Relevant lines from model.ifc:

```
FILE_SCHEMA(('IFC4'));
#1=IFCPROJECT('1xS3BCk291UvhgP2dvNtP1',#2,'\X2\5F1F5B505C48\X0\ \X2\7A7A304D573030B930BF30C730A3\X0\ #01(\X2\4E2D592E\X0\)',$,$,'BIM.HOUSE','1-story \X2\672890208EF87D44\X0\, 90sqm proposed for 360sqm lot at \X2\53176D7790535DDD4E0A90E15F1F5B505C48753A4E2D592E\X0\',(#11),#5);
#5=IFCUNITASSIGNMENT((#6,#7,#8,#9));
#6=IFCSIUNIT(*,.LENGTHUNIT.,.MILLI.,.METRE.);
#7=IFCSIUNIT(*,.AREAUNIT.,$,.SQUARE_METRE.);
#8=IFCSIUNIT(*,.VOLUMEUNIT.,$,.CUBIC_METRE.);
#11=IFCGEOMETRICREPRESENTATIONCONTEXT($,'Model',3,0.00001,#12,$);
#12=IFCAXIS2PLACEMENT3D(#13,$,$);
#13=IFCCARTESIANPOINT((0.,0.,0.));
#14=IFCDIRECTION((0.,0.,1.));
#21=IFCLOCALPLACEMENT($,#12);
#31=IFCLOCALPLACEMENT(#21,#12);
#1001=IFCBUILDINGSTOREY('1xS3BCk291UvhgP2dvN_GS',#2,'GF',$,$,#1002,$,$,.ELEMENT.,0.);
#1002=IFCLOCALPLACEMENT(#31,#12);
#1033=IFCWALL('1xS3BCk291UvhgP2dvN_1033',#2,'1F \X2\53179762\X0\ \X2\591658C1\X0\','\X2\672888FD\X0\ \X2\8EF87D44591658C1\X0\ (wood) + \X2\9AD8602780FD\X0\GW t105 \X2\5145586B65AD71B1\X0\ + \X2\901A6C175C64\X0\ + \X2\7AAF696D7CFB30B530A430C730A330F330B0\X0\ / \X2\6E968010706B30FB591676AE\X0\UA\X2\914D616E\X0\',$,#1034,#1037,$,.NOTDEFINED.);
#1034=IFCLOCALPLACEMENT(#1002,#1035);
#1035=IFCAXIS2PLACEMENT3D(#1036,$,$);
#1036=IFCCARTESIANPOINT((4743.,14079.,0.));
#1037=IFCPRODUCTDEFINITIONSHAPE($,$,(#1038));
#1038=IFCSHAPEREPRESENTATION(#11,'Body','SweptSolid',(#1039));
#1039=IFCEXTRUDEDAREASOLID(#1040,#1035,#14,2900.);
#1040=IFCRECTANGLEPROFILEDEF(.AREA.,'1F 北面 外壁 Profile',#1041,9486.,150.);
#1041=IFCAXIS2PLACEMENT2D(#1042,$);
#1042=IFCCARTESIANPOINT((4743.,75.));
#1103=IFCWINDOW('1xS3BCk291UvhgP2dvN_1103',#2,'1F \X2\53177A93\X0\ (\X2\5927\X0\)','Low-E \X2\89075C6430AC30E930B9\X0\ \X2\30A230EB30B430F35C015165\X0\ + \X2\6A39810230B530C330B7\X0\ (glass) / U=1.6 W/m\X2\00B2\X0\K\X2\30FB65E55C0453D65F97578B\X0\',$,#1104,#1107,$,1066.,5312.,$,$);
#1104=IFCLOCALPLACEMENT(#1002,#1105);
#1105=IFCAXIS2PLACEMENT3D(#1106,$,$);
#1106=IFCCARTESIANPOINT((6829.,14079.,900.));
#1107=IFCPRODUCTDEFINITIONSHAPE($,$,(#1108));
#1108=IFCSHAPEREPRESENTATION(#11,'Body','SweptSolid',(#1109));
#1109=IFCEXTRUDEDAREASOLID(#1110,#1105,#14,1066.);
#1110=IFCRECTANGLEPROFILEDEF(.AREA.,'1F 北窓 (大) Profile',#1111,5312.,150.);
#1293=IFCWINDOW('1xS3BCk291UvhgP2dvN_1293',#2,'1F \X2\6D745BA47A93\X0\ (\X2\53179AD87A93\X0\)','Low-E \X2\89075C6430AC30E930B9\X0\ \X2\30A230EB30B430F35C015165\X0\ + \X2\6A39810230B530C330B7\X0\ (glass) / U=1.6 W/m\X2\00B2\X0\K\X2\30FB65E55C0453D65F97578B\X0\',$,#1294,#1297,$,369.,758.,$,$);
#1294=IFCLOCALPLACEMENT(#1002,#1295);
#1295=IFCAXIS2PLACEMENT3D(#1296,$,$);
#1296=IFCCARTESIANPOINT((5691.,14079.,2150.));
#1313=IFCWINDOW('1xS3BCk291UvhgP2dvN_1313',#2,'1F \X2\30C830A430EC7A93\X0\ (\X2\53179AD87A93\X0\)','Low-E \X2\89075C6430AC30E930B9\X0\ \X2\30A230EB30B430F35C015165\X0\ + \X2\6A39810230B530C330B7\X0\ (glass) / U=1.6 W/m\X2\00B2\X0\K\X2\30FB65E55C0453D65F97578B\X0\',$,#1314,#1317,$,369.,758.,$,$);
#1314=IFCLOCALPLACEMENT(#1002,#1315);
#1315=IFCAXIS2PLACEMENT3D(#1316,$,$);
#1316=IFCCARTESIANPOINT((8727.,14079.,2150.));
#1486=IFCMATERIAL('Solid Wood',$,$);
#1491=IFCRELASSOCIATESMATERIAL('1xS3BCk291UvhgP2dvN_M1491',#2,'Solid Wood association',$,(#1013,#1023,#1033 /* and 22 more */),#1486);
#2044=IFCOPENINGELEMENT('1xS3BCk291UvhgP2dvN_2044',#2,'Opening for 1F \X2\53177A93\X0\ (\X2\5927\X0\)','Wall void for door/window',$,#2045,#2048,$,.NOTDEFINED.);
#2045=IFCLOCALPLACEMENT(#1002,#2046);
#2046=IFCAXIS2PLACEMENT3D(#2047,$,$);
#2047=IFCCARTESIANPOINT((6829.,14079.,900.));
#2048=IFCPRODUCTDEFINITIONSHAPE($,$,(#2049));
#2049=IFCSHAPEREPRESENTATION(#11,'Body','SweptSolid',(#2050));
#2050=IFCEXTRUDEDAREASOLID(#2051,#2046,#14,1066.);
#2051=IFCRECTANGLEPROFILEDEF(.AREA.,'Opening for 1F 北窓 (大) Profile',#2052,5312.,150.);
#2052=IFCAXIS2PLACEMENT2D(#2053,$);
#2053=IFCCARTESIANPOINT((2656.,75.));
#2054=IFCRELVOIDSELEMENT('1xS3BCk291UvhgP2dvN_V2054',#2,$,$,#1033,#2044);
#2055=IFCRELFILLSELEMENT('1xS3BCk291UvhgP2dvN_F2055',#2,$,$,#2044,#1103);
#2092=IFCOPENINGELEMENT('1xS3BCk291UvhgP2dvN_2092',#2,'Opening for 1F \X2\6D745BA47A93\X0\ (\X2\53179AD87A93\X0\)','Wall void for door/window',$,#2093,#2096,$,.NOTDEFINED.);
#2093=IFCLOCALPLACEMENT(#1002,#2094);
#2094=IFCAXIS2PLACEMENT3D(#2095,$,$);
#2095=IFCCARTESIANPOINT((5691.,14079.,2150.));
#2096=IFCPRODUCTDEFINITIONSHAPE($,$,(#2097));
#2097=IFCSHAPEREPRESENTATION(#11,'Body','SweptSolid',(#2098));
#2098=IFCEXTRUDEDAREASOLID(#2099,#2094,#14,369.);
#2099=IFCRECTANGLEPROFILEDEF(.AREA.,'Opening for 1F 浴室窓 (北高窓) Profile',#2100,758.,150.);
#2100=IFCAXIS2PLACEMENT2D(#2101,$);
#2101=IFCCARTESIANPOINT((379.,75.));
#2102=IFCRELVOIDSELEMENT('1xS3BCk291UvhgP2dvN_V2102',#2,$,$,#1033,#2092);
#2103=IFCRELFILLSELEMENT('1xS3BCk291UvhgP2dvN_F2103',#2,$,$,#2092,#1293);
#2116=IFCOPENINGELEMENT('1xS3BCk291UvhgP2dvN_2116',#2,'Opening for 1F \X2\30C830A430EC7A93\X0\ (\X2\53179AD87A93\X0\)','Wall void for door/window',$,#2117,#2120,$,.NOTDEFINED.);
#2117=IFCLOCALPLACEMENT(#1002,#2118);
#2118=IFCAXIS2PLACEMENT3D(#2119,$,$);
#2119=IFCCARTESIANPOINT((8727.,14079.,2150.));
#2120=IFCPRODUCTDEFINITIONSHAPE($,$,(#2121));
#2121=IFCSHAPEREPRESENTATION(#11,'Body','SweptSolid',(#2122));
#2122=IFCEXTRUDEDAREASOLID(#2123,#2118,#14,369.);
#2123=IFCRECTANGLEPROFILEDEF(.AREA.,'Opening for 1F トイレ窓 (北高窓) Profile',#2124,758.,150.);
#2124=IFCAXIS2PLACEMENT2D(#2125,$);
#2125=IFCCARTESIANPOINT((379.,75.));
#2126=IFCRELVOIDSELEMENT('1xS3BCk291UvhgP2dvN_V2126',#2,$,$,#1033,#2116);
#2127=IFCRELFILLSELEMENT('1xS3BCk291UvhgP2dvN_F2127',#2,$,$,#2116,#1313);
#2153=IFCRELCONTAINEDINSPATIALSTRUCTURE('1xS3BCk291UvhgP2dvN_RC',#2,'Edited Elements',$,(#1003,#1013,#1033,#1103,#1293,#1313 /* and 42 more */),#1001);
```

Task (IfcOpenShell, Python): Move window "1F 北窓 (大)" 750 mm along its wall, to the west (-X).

```python
import ifcopenshell
import ifcopenshell.api.geometry
import ifcopenshell.util.placement
import ifcopenshell.util.unit

model = ifcopenshell.open("model.ifc")
unit_scale = ifcopenshell.util.unit.calculate_unit_scale(model)

window = model.by_guid("1xS3BCk291UvhgP2dvN_1103")
opening = window.FillsVoids[0].RelatingOpeningElement
wall = opening.VoidsElements[0].RelatingBuildingElement

wall_matrix = ifcopenshell.util.placement.get_local_placement(wall.ObjectPlacement)
shift = wall_matrix[:3, 0] * -0.75 / unit_scale
before = ifcopenshell.util.placement.get_local_placement(window.ObjectPlacement)[:3, 3].copy()

# The window is not placed relative to its opening, so move both.
for product in (opening, window):
    matrix = ifcopenshell.util.placement.get_local_placement(product.ObjectPlacement)
    matrix[:3, 3] += shift
    ifcopenshell.api.geometry.edit_object_placement(model, product=product, matrix=matrix, is_si=False)

after = ifcopenshell.util.placement.get_local_placement(window.ObjectPlacement)[:3, 3]
print("window moved by", (after - before).round(3) + 0.0)

model.write("model_edited.ifc")
```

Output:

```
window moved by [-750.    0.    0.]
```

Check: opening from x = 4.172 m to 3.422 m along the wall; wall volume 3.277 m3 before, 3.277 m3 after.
